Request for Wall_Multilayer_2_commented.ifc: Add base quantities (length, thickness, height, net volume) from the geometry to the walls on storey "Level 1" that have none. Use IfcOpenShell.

First a look at what the model holds.

```python
import ifcopenshell
import ifcopenshell.util.element
import ifcopenshell.util.unit

model = ifcopenshell.open("Wall_Multilayer_2_commented.ifc")
print(model.schema)
for unit_type in ("LENGTHUNIT", "AREAUNIT", "VOLUMEUNIT"):
    print(unit_type, ifcopenshell.util.unit.calculate_unit_scale(model, unit_type))
storey = next(s for s in model.by_type("IfcBuildingStorey") if s.Name == "Level 1")
walls = [e for e in ifcopenshell.util.element.get_decomposition(storey) if e.is_a("IfcWall")]
for e in sorted(walls, key=lambda e: e.id()):
    print(e.id(), e.is_a(), e.Name, list(ifcopenshell.util.element.get_psets(e, qtos_only=True)), sep=" | ")
```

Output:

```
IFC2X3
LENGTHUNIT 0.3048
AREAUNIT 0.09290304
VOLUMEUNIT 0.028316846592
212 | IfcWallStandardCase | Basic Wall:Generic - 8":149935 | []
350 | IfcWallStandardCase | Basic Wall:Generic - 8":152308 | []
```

```python
import ifcopenshell
import ifcopenshell.api.pset
import ifcopenshell.geom
import ifcopenshell.util.element
import ifcopenshell.util.shape
import ifcopenshell.util.unit

model = ifcopenshell.open("Wall_Multilayer_2_commented.ifc")
unit_scale = ifcopenshell.util.unit.calculate_unit_scale(model)
volume_scale = ifcopenshell.util.unit.calculate_unit_scale(model, "VOLUMEUNIT")
settings = ifcopenshell.geom.settings()

storey = next(s for s in model.by_type("IfcBuildingStorey") if s.Name == "Level 1")
walls = [e for e in ifcopenshell.util.element.get_decomposition(storey) if e.is_a("IfcWall")]

for e in sorted(walls, key=lambda e: e.id()):
    if ifcopenshell.util.element.get_psets(e, qtos_only=True, should_inherit=False):
        continue
    # Geometry comes back in metres, in the element's own axes.
    shape = ifcopenshell.geom.create_shape(settings, e)
    values = {
        "Length": ifcopenshell.util.shape.get_x(shape.geometry) / unit_scale,
        "Width": ifcopenshell.util.shape.get_y(shape.geometry) / unit_scale,
        "Height": ifcopenshell.util.shape.get_z(shape.geometry) / unit_scale,
        "NetVolume": ifcopenshell.util.shape.get_volume(shape.geometry) / volume_scale,
    }
    qto = ifcopenshell.api.pset.add_qto(model, product=e, name="BaseQuantities")
    ifcopenshell.api.pset.edit_qto(model, qto=qto, properties=values)
    print(e.id(), {k: round(v, 3) for k, v in values.items()})

model.write("Wall_Multilayer_2_commented-out.ifc")
```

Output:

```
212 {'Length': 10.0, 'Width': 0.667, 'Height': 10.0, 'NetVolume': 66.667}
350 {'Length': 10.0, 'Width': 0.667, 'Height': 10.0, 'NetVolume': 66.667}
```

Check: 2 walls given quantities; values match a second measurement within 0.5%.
